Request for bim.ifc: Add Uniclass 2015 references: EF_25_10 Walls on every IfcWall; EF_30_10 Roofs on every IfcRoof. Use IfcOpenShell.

First a look at what the model holds.

```python
import ifcopenshell

model = ifcopenshell.open("bim.ifc")
print(model.schema)
print("classifications:", [c.Name for c in model.by_type("IfcClassification")])
for ifc_class in ("IfcDoor", "IfcRoof", "IfcStair", "IfcWall", "IfcWindow"):
    print(ifc_class, len(model.by_type(ifc_class)))
```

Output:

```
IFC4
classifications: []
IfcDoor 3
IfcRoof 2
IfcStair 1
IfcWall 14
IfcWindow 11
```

```python
import ifcopenshell
import ifcopenshell.api.classification

model = ifcopenshell.open("bim.ifc")

system = ifcopenshell.api.classification.add_classification(model, classification="Uniclass 2015")

codes = {
    "IfcWall": ("EF_25_10", "Walls"),
    "IfcRoof": ("EF_30_10", "Roofs"),
}
for ifc_class, (code, name) in codes.items():
    products = model.by_type(ifc_class)
    ifcopenshell.api.classification.add_reference(
        model, products=products, classification=system, identification=code, name=name
    )
    print(code, len(products))

model.write("bim_updated.ifc")
```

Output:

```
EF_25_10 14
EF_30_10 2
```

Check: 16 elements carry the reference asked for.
